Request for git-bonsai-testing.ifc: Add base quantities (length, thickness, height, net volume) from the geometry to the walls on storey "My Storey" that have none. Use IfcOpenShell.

First a look at what the model holds.

```python
import ifcopenshell
import ifcopenshell.util.element
import ifcopenshell.util.unit

model = ifcopenshell.open("git-bonsai-testing.ifc")
print(model.schema)
for unit_type in ("LENGTHUNIT", "AREAUNIT", "VOLUMEUNIT"):
    print(unit_type, ifcopenshell.util.unit.calculate_unit_scale(model, unit_type))
storey = next(s for s in model.by_type("IfcBuildingStorey") if s.Name == "My Storey")
walls = [e for e in ifcopenshell.util.element.get_decomposition(storey) if e.is_a("IfcWall")]
for e in sorted(walls, key=lambda e: e.id()):
    print(e.id(), e.is_a(), e.Name, list(ifcopenshell.util.element.get_psets(e, qtos_only=True)), sep=" | ")
```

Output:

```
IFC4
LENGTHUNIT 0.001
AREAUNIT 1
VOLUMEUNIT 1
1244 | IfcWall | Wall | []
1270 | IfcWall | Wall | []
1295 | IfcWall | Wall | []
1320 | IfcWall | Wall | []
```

```python
import ifcopenshell
import ifcopenshell.api.pset
import ifcopenshell.geom
import ifcopenshell.util.element
import ifcopenshell.util.shape
import ifcopenshell.util.unit

model = ifcopenshell.open("git-bonsai-testing.ifc")
unit_scale = ifcopenshell.util.unit.calculate_unit_scale(model)
volume_scale = ifcopenshell.util.unit.calculate_unit_scale(model, "VOLUMEUNIT")
settings = ifcopenshell.geom.settings()

storey = next(s for s in model.by_type("IfcBuildingStorey") if s.Name == "My Storey")
walls = [e for e in ifcopenshell.util.element.get_decomposition(storey) if e.is_a("IfcWall")]

for e in sorted(walls, key=lambda e: e.id()):
    if ifcopenshell.util.element.get_psets(e, qtos_only=True, should_inherit=False):
        continue
    # Geometry comes back in metres, in the element's own axes.
    shape = ifcopenshell.geom.create_shape(settings, e)
    values = {
        "Length": ifcopenshell.util.shape.get_x(shape.geometry) / unit_scale,
        "Width": ifcopenshell.util.shape.get_y(shape.geometry) / unit_scale,
        "Height": ifcopenshell.util.shape.get_z(shape.geometry) / unit_scale,
        "NetVolume": ifcopenshell.util.shape.get_volume(shape.geometry) / volume_scale,
    }
    qto = ifcopenshell.api.pset.add_qto(model, product=e, name="Qto_WallBaseQuantities")
    ifcopenshell.api.pset.edit_qto(model, qto=qto, properties=values)
    print(e.id(), {k: round(v, 3) for k, v in values.items()})

model.write("git-bonsai-testing_v2.ifc")
```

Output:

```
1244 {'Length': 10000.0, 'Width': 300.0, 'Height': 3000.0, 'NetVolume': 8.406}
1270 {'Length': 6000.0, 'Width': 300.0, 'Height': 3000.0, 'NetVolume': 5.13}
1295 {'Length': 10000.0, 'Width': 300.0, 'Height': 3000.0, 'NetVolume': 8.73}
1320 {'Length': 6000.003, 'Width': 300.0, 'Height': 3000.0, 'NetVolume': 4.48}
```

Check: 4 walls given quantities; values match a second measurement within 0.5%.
